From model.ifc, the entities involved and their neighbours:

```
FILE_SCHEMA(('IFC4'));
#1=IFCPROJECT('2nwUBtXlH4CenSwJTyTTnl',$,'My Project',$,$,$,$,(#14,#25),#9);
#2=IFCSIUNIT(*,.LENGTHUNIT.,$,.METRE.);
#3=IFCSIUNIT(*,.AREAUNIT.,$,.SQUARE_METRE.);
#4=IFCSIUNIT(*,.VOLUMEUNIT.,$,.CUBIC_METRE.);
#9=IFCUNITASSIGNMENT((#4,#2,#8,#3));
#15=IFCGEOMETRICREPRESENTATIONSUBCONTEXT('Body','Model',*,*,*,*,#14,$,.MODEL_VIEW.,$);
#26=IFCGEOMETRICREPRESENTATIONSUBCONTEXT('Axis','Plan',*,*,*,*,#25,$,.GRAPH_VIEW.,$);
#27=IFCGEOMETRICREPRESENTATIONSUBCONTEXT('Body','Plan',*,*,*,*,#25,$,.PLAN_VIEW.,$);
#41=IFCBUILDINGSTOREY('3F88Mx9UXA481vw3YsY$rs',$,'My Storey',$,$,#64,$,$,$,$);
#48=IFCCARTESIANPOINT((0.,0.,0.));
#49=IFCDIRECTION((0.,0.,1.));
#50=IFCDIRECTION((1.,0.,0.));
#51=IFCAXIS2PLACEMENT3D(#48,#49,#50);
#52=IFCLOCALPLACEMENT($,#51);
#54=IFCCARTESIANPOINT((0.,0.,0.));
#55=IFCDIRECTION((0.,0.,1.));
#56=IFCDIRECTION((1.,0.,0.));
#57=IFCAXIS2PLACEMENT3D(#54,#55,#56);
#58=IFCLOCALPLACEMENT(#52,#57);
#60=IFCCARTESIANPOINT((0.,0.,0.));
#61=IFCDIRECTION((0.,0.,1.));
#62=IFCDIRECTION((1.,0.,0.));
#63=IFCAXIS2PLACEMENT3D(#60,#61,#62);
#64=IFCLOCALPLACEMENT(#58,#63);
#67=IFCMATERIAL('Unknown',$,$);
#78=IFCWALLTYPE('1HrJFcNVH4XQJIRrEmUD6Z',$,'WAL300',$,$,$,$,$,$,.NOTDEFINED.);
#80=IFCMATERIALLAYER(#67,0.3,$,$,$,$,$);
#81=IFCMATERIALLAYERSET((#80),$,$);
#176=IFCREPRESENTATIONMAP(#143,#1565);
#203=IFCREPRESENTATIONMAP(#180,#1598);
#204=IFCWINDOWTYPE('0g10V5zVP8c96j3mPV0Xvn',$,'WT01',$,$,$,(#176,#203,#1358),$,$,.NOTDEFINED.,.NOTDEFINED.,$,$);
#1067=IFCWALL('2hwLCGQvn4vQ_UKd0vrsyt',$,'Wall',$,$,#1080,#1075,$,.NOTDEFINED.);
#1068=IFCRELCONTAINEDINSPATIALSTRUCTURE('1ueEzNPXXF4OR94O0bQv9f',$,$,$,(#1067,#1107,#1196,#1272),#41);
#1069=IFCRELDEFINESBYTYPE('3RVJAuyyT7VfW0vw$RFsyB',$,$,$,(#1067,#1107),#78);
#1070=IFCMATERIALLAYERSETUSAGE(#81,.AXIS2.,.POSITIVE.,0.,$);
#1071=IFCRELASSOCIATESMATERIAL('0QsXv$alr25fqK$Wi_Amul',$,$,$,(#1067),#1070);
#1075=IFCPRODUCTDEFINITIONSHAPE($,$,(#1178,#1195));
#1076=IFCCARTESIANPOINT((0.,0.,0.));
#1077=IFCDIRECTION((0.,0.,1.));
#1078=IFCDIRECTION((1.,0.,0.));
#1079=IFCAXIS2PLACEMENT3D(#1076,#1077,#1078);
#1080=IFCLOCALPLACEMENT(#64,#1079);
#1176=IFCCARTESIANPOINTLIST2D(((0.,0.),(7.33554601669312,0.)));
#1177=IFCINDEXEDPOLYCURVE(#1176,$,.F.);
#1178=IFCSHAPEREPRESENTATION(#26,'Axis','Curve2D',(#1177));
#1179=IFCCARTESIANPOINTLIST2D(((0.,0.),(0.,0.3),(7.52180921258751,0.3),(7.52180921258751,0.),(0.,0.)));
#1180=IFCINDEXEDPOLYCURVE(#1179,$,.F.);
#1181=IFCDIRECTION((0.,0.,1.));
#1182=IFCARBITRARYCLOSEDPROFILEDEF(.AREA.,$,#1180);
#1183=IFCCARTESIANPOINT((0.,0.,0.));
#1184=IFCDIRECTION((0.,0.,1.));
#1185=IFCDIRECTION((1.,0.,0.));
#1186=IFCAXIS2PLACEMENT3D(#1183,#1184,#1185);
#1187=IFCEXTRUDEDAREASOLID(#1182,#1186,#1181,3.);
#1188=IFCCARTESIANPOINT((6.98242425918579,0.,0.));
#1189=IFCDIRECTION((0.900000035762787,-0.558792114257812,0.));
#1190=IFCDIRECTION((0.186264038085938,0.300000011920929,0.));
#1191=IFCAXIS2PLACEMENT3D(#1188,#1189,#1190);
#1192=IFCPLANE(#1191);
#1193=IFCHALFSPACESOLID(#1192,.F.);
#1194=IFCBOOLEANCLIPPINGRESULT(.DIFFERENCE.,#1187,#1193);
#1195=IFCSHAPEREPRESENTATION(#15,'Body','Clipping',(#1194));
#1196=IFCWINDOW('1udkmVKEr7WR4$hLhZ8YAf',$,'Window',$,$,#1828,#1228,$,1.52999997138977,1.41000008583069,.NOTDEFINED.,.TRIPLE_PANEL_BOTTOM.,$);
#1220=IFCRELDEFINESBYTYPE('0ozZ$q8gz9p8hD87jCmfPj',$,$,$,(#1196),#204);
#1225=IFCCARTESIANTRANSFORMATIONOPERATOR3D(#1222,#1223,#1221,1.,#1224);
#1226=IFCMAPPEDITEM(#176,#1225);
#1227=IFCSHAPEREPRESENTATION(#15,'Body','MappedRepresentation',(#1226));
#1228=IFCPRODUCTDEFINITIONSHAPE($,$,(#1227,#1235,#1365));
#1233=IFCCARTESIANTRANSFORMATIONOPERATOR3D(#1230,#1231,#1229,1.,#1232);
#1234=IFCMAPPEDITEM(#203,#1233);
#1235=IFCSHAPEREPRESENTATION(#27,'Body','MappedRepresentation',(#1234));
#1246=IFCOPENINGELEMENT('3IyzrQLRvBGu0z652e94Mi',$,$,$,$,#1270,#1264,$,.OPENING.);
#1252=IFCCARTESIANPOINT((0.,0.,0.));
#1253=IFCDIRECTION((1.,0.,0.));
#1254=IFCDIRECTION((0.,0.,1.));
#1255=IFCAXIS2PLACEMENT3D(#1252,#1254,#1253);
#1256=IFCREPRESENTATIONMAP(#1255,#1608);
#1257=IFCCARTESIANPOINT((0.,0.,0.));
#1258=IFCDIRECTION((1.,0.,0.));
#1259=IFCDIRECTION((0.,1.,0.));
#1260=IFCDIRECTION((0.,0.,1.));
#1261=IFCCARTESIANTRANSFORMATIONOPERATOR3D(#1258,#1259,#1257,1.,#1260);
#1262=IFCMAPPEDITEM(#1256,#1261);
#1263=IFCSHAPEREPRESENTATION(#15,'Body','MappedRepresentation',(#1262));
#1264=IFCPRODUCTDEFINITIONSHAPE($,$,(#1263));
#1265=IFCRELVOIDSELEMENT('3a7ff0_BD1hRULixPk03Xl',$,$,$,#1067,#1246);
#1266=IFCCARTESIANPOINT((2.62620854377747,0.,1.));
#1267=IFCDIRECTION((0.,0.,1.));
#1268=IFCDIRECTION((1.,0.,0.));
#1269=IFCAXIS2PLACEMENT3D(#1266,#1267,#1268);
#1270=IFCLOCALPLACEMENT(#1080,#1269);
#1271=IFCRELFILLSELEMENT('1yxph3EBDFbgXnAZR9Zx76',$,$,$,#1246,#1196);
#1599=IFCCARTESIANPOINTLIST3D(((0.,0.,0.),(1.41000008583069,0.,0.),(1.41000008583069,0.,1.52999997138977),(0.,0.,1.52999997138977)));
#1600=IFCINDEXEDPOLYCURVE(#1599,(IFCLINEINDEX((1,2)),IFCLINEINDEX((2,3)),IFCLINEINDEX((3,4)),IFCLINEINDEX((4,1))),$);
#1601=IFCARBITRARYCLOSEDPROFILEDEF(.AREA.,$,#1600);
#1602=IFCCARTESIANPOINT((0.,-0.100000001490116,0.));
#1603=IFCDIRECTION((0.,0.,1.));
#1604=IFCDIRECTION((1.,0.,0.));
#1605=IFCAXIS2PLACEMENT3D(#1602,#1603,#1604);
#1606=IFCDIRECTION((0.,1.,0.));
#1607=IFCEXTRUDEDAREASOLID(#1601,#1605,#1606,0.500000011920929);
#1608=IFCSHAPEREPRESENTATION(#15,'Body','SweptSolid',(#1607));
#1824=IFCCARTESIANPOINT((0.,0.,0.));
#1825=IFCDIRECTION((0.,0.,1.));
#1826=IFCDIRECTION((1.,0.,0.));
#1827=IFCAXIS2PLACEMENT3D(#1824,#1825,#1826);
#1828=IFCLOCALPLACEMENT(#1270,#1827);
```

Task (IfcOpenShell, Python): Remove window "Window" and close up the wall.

```python
import ifcopenshell
import ifcopenshell.api.feature
import ifcopenshell.api.root
import ifcopenshell.geom
import ifcopenshell.util.shape

model = ifcopenshell.open("model.ifc")
settings = ifcopenshell.geom.settings()


def volume(element):
    """Net volume in cubic metres, openings subtracted."""
    shape = ifcopenshell.geom.create_shape(settings, element)
    return ifcopenshell.util.shape.get_volume(shape.geometry)


window = model.by_guid("1udkmVKEr7WR4$hLhZ8YAf")
opening = window.FillsVoids[0].RelatingOpeningElement
wall = opening.VoidsElements[0].RelatingBuildingElement
before = volume(wall)

ifcopenshell.api.root.remove_product(model, product=window)
ifcopenshell.api.feature.remove_feature(model, feature=opening)

after = volume(wall)

print(f"wall volume {before:.3f} -> {after:.3f} m3")

model.write("model_rev.ifc")
```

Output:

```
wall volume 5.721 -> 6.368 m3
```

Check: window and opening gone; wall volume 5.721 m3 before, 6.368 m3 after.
